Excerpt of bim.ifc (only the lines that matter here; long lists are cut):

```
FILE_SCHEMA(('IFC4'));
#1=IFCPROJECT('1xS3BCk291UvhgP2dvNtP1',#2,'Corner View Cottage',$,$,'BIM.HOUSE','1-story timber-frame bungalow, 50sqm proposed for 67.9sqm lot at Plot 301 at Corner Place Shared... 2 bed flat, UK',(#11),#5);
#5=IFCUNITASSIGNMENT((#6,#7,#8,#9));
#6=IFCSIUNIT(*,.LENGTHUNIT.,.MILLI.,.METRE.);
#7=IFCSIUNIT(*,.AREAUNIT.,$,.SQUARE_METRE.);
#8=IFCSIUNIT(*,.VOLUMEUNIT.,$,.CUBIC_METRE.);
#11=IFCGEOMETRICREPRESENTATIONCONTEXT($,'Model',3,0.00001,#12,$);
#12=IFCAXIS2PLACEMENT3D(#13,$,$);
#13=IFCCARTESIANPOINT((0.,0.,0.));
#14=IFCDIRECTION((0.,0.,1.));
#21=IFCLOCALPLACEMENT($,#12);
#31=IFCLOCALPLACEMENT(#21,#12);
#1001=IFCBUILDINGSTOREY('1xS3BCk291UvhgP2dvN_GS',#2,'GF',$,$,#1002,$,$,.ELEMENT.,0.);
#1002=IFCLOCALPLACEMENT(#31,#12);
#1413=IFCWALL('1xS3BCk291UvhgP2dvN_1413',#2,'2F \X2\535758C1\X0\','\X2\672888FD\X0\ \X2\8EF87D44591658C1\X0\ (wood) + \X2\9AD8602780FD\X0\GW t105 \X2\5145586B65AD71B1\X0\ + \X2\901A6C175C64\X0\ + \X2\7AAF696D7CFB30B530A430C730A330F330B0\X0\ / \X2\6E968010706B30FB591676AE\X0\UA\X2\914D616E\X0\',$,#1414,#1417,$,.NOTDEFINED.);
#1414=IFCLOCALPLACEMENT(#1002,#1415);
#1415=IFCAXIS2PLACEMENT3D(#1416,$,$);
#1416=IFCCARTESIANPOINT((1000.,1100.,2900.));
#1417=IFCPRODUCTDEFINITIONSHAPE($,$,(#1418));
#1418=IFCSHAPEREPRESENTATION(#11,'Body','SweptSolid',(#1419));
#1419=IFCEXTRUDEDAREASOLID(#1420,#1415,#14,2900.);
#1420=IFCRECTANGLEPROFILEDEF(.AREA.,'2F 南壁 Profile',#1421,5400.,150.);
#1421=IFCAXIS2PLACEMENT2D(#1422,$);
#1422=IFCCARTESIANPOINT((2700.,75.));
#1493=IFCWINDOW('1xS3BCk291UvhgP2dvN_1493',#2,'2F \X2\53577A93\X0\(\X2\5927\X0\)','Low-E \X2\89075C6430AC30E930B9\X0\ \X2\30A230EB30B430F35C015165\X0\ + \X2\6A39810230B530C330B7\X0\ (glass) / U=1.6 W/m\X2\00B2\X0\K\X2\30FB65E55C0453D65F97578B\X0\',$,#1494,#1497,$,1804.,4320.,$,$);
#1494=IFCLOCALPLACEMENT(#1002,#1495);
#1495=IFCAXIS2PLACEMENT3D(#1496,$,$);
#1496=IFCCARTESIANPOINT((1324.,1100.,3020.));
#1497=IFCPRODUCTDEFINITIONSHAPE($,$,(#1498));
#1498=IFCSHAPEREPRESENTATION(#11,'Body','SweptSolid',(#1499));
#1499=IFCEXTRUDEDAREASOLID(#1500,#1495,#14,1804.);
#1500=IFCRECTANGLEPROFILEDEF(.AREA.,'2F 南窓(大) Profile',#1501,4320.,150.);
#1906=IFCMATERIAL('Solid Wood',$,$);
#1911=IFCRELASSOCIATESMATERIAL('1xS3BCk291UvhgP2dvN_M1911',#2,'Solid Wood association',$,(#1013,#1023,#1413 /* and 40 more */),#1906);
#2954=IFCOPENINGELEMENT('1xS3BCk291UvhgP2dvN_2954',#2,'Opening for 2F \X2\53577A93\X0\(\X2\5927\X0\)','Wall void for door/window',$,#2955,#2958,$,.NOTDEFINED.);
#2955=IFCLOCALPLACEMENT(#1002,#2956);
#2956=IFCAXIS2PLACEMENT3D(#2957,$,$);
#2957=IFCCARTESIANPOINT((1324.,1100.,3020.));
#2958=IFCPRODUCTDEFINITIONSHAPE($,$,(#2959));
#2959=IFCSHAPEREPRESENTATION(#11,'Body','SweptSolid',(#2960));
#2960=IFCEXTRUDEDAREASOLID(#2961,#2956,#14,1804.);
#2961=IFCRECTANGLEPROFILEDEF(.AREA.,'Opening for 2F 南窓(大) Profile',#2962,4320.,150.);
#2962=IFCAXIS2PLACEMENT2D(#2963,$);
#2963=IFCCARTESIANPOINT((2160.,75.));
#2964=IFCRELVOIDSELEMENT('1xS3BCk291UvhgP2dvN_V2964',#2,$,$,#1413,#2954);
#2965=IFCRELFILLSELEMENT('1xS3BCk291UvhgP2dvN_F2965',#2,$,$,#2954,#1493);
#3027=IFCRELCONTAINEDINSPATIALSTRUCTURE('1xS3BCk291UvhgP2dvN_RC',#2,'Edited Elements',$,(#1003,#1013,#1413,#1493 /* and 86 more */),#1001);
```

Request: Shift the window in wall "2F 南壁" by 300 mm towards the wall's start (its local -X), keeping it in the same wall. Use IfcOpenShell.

```python
import ifcopenshell
import ifcopenshell.api.geometry
import ifcopenshell.util.placement
import ifcopenshell.util.unit

model = ifcopenshell.open("bim.ifc")
unit_scale = ifcopenshell.util.unit.calculate_unit_scale(model)

window = model.by_guid("1xS3BCk291UvhgP2dvN_1493")
opening = window.FillsVoids[0].RelatingOpeningElement
wall = opening.VoidsElements[0].RelatingBuildingElement

wall_matrix = ifcopenshell.util.placement.get_local_placement(wall.ObjectPlacement)
shift = wall_matrix[:3, 0] * -0.3 / unit_scale
before = ifcopenshell.util.placement.get_local_placement(window.ObjectPlacement)[:3, 3].copy()

# The window is not placed relative to its opening, so move both.
for product in (opening, window):
    matrix = ifcopenshell.util.placement.get_local_placement(product.ObjectPlacement)
    matrix[:3, 3] += shift
    ifcopenshell.api.geometry.edit_object_placement(model, product=product, matrix=matrix, is_si=False)

after = ifcopenshell.util.placement.get_local_placement(window.ObjectPlacement)[:3, 3]
print("window moved by", (after - before).round(3) + 0.0)

model.write("bim_rev.ifc")
```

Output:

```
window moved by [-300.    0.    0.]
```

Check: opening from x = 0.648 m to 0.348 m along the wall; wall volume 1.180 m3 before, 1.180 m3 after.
